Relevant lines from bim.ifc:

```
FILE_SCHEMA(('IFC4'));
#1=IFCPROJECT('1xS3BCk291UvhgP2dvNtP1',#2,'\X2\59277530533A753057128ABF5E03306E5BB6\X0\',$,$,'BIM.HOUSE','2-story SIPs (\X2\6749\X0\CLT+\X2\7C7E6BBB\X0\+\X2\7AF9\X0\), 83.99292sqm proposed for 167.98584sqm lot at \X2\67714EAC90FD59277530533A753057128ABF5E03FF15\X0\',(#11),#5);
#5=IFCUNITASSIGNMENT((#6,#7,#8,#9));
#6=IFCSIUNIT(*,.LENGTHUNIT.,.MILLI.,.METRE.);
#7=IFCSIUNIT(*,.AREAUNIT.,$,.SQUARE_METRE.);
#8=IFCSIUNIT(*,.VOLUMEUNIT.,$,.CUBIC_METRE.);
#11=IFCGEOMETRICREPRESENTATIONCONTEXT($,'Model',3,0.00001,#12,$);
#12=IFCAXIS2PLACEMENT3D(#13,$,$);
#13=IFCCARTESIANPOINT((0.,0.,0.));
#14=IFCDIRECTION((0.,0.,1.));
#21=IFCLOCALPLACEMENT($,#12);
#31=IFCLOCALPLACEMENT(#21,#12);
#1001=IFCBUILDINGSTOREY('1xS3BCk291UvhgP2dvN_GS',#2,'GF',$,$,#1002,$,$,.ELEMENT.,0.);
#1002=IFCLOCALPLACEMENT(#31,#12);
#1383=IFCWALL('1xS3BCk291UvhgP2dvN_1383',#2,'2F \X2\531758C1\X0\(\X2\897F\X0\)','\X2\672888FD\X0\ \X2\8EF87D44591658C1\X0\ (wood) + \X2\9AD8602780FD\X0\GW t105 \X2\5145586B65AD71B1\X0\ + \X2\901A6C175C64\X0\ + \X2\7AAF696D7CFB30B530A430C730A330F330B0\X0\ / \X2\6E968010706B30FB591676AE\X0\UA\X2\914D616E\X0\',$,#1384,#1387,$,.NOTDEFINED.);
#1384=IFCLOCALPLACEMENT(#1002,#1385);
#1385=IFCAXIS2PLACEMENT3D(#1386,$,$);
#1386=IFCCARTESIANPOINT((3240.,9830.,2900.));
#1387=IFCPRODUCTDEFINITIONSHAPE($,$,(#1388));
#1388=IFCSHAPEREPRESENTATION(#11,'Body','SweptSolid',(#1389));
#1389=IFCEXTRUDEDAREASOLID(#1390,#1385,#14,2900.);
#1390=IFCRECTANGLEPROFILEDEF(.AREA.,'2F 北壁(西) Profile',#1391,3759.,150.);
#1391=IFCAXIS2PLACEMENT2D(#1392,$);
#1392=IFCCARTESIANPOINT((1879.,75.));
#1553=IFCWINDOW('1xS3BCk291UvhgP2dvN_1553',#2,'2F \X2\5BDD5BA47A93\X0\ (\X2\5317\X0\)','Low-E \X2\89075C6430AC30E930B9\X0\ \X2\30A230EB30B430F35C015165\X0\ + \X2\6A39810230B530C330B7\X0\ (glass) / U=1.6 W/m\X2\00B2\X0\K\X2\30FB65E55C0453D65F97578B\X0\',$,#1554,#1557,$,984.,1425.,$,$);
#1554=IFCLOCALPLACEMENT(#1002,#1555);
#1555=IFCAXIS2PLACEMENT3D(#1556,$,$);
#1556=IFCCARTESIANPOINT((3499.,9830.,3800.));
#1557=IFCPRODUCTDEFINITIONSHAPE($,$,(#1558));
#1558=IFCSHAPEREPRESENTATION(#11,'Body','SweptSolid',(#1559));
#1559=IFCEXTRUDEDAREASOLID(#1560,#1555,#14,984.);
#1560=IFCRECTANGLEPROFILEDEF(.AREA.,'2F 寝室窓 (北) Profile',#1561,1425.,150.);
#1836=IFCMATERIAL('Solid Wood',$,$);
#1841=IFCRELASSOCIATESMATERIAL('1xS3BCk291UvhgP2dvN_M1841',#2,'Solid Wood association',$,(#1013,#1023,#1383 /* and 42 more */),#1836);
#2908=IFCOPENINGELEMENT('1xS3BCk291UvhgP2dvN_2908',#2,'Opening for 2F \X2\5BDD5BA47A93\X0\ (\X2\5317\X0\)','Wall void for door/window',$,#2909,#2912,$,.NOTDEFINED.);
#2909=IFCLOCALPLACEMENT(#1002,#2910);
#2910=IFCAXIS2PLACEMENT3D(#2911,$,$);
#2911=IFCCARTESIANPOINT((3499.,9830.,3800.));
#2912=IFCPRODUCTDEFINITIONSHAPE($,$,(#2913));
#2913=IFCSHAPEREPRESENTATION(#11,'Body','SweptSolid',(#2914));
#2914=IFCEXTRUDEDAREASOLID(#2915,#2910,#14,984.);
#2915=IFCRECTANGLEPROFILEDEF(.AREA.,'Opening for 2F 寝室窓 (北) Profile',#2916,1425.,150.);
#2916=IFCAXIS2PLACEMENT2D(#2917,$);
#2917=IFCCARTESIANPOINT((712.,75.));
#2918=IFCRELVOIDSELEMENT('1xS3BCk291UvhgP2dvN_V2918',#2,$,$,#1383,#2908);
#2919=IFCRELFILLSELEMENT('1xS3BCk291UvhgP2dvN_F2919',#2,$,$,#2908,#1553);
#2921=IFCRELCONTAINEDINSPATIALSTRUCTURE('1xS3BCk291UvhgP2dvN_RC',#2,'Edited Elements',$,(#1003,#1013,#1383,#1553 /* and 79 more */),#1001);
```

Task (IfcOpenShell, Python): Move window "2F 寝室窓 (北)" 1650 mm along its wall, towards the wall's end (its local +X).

```python
import ifcopenshell
import ifcopenshell.api.geometry
import ifcopenshell.util.placement
import ifcopenshell.util.unit

model = ifcopenshell.open("bim.ifc")
unit_scale = ifcopenshell.util.unit.calculate_unit_scale(model)

window = model.by_guid("1xS3BCk291UvhgP2dvN_1553")
opening = window.FillsVoids[0].RelatingOpeningElement
wall = opening.VoidsElements[0].RelatingBuildingElement

wall_matrix = ifcopenshell.util.placement.get_local_placement(wall.ObjectPlacement)
shift = wall_matrix[:3, 0] * 1.65 / unit_scale
before = ifcopenshell.util.placement.get_local_placement(window.ObjectPlacement)[:3, 3].copy()

# The window is not placed relative to its opening, so move both.
for product in (opening, window):
    matrix = ifcopenshell.util.placement.get_local_placement(product.ObjectPlacement)
    matrix[:3, 3] += shift
    ifcopenshell.api.geometry.edit_object_placement(model, product=product, matrix=matrix, is_si=False)

after = ifcopenshell.util.placement.get_local_placement(window.ObjectPlacement)[:3, 3]
print("window moved by", (after - before).round(3) + 0.0)

model.write("bim_updated.ifc")
```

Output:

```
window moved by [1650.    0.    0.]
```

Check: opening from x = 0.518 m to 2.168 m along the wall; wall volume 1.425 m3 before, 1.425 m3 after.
